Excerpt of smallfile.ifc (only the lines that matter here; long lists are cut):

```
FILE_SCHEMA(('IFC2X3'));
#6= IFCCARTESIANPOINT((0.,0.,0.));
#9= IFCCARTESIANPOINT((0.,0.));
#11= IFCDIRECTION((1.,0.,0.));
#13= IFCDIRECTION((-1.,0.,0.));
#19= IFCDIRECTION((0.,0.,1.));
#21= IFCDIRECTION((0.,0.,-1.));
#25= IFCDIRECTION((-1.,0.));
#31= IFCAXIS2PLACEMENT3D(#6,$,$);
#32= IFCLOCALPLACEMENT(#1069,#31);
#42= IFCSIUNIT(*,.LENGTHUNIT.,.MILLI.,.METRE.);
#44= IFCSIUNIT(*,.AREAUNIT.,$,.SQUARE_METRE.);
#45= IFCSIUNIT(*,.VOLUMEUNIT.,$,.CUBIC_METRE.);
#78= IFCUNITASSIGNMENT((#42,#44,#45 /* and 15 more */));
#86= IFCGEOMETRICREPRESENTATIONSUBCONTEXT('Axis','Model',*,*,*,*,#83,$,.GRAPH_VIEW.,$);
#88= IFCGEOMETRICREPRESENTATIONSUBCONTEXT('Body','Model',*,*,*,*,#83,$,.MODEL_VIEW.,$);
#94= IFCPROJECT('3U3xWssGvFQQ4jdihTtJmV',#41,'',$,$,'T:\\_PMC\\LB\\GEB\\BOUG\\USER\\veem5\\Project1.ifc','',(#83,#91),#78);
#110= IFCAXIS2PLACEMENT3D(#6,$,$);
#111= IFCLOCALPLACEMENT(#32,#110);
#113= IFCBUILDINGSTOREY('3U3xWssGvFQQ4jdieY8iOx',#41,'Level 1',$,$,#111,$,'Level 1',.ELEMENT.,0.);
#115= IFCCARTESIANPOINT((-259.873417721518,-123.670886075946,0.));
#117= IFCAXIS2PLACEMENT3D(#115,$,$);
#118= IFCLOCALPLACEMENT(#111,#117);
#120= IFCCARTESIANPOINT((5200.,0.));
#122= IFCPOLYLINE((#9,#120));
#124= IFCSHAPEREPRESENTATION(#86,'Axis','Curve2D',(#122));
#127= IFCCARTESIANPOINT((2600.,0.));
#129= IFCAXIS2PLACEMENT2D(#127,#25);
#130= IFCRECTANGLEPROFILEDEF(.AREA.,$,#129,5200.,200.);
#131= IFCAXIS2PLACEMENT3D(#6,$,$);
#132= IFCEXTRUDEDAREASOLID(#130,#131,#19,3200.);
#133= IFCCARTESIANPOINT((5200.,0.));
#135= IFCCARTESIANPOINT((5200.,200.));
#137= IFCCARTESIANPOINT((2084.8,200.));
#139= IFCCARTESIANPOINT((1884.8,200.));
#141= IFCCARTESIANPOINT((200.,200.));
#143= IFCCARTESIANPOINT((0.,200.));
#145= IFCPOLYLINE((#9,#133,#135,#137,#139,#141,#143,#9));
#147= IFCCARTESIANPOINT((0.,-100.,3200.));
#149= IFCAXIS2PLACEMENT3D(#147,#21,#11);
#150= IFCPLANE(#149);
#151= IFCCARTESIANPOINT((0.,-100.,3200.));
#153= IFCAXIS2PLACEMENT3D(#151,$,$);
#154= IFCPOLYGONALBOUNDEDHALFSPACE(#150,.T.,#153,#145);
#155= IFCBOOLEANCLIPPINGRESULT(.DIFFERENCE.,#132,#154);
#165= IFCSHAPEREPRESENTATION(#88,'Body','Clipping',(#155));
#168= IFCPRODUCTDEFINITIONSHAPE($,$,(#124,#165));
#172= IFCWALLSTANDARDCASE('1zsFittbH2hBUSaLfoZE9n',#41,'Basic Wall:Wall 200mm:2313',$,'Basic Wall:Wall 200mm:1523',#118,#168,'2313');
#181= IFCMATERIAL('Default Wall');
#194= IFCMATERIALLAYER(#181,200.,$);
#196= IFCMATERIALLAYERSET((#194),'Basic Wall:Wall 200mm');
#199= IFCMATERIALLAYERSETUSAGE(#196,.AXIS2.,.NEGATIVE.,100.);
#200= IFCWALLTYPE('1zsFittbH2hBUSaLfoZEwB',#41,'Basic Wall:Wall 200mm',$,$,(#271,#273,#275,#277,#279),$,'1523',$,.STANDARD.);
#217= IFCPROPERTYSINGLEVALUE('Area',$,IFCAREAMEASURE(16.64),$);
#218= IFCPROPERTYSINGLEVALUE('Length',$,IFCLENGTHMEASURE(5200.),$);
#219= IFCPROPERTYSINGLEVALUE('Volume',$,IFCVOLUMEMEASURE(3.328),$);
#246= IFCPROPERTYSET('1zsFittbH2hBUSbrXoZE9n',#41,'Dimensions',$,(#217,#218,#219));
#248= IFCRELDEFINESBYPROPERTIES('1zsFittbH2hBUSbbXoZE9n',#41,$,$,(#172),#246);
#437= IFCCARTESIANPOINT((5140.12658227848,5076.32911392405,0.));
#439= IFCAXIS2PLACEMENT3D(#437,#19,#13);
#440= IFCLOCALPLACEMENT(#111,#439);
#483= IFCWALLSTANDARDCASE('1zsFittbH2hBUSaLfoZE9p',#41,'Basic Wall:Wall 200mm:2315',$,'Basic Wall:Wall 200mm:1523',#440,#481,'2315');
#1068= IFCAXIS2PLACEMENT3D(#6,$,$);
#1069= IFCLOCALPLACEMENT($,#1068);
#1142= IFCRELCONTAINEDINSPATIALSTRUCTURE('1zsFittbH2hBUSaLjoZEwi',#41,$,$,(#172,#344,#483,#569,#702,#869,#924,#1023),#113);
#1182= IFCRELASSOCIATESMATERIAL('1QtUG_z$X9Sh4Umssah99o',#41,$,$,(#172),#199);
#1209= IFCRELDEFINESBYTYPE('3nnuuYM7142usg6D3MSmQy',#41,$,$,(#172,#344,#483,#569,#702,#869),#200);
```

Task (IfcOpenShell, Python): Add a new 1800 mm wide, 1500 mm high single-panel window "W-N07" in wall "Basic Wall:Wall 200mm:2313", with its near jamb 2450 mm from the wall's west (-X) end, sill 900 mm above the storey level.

```python
import numpy as np
import ifcopenshell
import ifcopenshell.api.feature
import ifcopenshell.api.geometry
import ifcopenshell.api.pset
import ifcopenshell.api.root
import ifcopenshell.api.spatial
import ifcopenshell.api.type
import ifcopenshell.geom
import ifcopenshell.util.element
import ifcopenshell.util.placement
import ifcopenshell.util.representation
import ifcopenshell.util.shape
import ifcopenshell.util.unit

model = ifcopenshell.open("smallfile.ifc")
unit_scale = ifcopenshell.util.unit.calculate_unit_scale(model)
area_scale = ifcopenshell.util.unit.calculate_unit_scale(model, "AREAUNIT")
volume_scale = ifcopenshell.util.unit.calculate_unit_scale(model, "VOLUMEUNIT")
settings = ifcopenshell.geom.settings()


def volume(element):
    """Net volume in cubic metres, openings subtracted."""
    shape = ifcopenshell.geom.create_shape(settings, element)
    return ifcopenshell.util.shape.get_volume(shape.geometry)


wall = model.by_id(172)
storey = ifcopenshell.util.element.get_container(wall, ifc_class="IfcBuildingStorey")
context = ifcopenshell.util.representation.get_context(model, "Model", "Body", "MODEL_VIEW")
before = volume(wall)

width, height, from_end, sill = 1.8, 1.5, 2.45, 0.9  # metres

# The wall runs along its own X axis, and the end named is its -X end.
wall_shape = ifcopenshell.geom.create_shape(settings, wall)
x, y, z = ifcopenshell.util.shape.get_vertices(wall_shape.geometry).T
start = x.min() + from_end
face, thickness = float(y.min()), float(y.max() - y.min())
wall_matrix = ifcopenshell.util.placement.get_local_placement(wall.ObjectPlacement)
level = ifcopenshell.util.placement.get_local_placement(storey.ObjectPlacement)[2, 3]


def in_wall(x, y):
    """Placement at x, y metres in the wall's axes, at sill height."""
    matrix = wall_matrix.copy()
    matrix[:, 3] = wall_matrix @ np.array([x / unit_scale, y / unit_scale, 0.0, 1.0])
    matrix[2, 3] = level + sill / unit_scale
    return matrix


# Opening: a box that overshoots both wall faces by 50 mm.
opening = ifcopenshell.api.root.create_entity(model, ifc_class="IfcOpeningElement")
box = ifcopenshell.api.geometry.add_wall_representation(
    model, context=context, length=width, height=height, thickness=thickness + 0.1
)
ifcopenshell.api.geometry.assign_representation(model, product=opening, representation=box)
ifcopenshell.api.geometry.edit_object_placement(model, product=opening, matrix=in_wall(start, face - 0.05), is_si=False)
ifcopenshell.api.feature.add_feature(model, feature=opening, element=wall)

window = ifcopenshell.api.root.create_entity(model, ifc_class="IfcWindow", name="W-N07")
window.OverallWidth, window.OverallHeight = width / unit_scale, height / unit_scale
body = ifcopenshell.api.geometry.add_window_representation(
    model,
    context=context,
    overall_width=window.OverallWidth,
    overall_height=window.OverallHeight,
    partition_type="SINGLE_PANEL",
)
ifcopenshell.api.geometry.assign_representation(model, product=window, representation=body)
ifcopenshell.api.spatial.assign_container(model, products=[window], relating_structure=storey)
fills = ifcopenshell.api.feature.add_filling(model, opening=opening, element=window)
fills.OwnerHistory = window.OwnerHistory  # required in IFC2X3

# IFC2X3 keeps the operation on the window style.
style = ifcopenshell.api.root.create_entity(model, ifc_class="IfcWindowStyle", name="W-N07")
style.OperationType, style.ConstructionType = "SINGLE_PANEL", "NOTDEFINED"
style.ParameterTakesPrecedence = style.Sizeable = False
ifcopenshell.api.type.assign_type(model, related_objects=[window], relating_type=style)

# Centre the window in the wall's thickness.
ifcopenshell.api.geometry.edit_object_placement(model, product=window, matrix=in_wall(start, face), is_si=False)
window_shape = ifcopenshell.geom.create_shape(settings, window)
depth = ifcopenshell.util.shape.get_vertices(window_shape.geometry)[:, 1]
offset = face + thickness / 2 - (depth.min() + depth.max()) / 2
ifcopenshell.api.geometry.edit_object_placement(model, product=window, matrix=in_wall(start, offset), is_si=False)

after = volume(wall)

# Update the wall's stored quantities.
pset = model.by_id(ifcopenshell.util.element.get_pset(wall, "Dimensions", should_inherit=False)["id"])
ifcopenshell.api.pset.edit_pset(model, pset=pset, properties={
    "Area": model.create_entity("IfcAreaMeasure", after / thickness / area_scale),
    "Volume": model.create_entity("IfcVolumeMeasure", after / volume_scale),
})

print(f"wall volume {before:.3f} -> {after:.3f} m3")

model.write("smallfile_updated.ifc")
```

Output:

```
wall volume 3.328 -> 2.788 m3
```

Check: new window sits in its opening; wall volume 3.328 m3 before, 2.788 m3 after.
